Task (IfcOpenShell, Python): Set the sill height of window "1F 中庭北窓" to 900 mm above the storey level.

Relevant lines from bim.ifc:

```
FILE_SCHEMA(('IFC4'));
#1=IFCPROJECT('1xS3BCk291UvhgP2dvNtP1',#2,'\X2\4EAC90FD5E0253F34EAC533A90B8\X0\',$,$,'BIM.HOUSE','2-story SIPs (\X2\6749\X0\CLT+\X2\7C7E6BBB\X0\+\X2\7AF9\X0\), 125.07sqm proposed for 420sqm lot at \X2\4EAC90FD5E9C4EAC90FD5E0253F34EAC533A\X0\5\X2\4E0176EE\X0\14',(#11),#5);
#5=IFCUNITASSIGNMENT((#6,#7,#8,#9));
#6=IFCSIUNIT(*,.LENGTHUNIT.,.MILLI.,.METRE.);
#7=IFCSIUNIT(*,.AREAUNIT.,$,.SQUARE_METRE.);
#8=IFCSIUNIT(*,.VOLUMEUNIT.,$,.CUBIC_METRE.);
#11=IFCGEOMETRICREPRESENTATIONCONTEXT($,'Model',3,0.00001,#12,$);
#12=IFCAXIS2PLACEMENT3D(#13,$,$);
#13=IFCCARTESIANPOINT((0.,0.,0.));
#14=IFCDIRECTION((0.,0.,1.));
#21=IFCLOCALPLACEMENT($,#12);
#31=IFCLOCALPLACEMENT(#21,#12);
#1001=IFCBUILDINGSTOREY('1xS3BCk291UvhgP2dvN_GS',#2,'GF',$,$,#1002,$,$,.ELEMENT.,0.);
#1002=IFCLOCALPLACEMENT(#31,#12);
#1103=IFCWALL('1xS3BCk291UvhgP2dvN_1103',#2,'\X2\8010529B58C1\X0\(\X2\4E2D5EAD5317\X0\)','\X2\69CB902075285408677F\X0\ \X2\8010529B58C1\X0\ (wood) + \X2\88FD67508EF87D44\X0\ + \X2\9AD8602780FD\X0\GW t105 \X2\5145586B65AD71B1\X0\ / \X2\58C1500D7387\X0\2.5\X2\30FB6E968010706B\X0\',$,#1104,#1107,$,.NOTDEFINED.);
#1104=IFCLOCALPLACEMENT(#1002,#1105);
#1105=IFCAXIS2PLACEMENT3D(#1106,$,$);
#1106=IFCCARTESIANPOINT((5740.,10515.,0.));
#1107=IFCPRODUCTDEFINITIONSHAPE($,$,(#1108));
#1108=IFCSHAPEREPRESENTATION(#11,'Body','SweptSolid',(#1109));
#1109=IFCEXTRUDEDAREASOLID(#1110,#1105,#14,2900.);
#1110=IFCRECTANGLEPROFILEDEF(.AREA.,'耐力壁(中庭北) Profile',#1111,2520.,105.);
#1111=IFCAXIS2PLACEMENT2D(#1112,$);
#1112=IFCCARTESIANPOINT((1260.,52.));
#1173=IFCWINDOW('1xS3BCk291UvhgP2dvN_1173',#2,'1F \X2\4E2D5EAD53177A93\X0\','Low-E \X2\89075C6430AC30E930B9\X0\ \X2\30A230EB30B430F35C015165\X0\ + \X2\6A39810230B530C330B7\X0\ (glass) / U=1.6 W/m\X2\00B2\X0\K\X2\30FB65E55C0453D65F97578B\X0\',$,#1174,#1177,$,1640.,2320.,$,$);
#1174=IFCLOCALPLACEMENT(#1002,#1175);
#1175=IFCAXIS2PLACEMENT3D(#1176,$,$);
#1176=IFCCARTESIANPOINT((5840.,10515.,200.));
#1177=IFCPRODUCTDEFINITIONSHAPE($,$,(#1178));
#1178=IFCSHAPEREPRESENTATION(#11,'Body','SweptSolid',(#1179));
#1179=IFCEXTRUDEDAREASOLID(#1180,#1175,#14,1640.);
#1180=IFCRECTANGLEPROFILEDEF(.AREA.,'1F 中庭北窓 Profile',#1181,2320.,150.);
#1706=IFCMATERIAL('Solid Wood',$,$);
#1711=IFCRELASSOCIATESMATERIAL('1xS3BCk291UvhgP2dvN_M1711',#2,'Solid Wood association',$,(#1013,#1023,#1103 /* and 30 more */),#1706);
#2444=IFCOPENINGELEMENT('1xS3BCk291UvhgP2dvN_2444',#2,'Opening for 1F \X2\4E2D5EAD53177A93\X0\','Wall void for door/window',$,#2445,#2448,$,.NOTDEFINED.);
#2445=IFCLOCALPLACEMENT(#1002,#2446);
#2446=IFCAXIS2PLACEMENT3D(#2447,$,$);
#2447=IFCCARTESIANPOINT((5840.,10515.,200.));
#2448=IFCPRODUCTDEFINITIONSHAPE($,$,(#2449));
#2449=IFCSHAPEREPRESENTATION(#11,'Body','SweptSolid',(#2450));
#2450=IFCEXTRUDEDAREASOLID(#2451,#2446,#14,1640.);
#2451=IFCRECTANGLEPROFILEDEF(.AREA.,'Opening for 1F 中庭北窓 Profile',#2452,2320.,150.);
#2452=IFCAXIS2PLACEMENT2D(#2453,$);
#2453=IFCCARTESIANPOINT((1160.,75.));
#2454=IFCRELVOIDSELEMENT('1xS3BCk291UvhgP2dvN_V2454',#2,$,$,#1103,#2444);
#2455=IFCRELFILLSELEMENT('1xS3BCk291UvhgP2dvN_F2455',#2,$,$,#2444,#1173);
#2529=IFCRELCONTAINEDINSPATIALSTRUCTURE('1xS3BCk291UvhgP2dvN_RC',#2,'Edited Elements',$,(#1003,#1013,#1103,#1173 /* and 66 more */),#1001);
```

```python
import numpy as np
import ifcopenshell
import ifcopenshell.api.geometry
import ifcopenshell.geom
import ifcopenshell.util.element
import ifcopenshell.util.placement
import ifcopenshell.util.shape
import ifcopenshell.util.unit

model = ifcopenshell.open("bim.ifc")
unit_scale = ifcopenshell.util.unit.calculate_unit_scale(model)

window = model.by_guid("1xS3BCk291UvhgP2dvN_1173")
opening = window.FillsVoids[0].RelatingOpeningElement
storey = ifcopenshell.util.element.get_container(window, ifc_class="IfcBuildingStorey")
level = ifcopenshell.util.placement.get_local_placement(storey.ObjectPlacement)[2, 3]

# The opening's origin need not be at the sill, so measure its lowest point.
shape = ifcopenshell.geom.create_shape(ifcopenshell.geom.settings(), opening)
bottom = ifcopenshell.util.shape.get_shape_bottom_elevation(shape, shape.geometry) / unit_scale
dz = level + 900.0 - bottom

shift = np.array([0.0, 0.0, dz])
# The window is not placed relative to its opening, so move both.
for product in (opening, window):
    matrix = ifcopenshell.util.placement.get_local_placement(product.ObjectPlacement)
    matrix[:3, 3] += shift
    ifcopenshell.api.geometry.edit_object_placement(model, product=product, matrix=matrix, is_si=False)

print(f"moved by {dz * unit_scale:+.3f} m")

model.write("bim_edited.ifc")
```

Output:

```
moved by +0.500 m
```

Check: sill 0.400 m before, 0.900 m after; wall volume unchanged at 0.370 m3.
